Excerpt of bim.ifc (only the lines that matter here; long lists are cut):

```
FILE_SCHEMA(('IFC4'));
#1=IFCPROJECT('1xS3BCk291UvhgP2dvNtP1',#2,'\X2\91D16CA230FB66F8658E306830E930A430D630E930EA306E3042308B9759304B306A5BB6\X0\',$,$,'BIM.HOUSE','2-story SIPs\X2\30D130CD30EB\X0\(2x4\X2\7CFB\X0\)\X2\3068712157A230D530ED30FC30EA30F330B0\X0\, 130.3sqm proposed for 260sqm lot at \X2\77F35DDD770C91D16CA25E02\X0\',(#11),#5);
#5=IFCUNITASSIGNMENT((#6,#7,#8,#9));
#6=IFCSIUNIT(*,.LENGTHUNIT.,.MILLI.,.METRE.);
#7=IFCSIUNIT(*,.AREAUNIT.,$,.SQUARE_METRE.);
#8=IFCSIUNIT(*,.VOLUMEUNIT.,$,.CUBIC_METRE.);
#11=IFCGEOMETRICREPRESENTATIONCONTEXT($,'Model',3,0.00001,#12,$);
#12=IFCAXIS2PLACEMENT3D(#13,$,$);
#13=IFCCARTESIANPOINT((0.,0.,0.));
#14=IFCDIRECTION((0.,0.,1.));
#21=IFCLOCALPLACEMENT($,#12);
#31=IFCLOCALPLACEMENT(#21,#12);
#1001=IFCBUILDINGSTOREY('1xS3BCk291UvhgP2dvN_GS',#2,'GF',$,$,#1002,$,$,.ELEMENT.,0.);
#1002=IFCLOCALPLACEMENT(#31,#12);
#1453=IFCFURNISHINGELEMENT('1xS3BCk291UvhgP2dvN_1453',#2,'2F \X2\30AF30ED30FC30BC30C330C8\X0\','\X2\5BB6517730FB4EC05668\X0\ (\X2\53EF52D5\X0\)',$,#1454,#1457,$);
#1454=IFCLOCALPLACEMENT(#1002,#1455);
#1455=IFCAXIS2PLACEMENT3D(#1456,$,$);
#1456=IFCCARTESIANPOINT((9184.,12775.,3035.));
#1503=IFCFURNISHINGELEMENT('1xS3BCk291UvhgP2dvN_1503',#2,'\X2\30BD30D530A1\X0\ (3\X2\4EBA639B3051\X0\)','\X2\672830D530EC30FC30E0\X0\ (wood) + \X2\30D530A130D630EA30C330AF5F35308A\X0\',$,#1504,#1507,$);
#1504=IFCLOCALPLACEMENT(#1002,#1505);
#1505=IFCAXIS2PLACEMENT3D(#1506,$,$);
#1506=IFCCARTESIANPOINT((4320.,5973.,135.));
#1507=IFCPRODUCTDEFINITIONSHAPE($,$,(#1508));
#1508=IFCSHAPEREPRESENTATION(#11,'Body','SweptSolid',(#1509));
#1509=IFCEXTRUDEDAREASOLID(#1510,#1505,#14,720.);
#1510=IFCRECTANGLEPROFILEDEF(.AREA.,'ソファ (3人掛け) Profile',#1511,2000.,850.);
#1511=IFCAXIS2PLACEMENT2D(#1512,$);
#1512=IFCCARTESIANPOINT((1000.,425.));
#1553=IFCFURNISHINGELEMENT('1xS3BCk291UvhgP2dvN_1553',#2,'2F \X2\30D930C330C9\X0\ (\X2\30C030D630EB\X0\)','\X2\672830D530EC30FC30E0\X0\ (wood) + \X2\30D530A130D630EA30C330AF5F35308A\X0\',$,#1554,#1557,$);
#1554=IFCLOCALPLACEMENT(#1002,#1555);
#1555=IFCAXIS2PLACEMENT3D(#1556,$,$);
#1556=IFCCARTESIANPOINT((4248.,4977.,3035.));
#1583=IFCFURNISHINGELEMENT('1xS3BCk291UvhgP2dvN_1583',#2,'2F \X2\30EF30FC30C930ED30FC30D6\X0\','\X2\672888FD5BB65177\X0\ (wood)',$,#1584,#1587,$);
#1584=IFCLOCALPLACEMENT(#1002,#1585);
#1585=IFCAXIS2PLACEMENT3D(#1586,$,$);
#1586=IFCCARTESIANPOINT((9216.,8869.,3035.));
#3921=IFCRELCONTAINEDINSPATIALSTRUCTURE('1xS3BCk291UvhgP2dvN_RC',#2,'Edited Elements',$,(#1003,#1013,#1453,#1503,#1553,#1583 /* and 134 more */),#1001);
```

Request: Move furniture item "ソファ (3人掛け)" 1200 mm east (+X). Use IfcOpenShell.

```python
import ifcopenshell
import ifcopenshell.api.geometry
import ifcopenshell.util.placement

model = ifcopenshell.open("bim.ifc")

item = model.by_id(1503)
matrix = ifcopenshell.util.placement.get_local_placement(item.ObjectPlacement)
matrix[0, 3] += 1200.0
ifcopenshell.api.geometry.edit_object_placement(model, product=item, matrix=matrix, is_si=False)

print(ifcopenshell.util.placement.get_local_placement(item.ObjectPlacement).round(3) + 0.0)

model.write("bim-out.ifc")
```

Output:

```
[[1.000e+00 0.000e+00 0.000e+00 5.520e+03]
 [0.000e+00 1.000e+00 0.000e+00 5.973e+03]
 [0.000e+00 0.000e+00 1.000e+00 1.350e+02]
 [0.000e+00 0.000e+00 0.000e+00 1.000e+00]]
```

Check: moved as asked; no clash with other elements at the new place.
